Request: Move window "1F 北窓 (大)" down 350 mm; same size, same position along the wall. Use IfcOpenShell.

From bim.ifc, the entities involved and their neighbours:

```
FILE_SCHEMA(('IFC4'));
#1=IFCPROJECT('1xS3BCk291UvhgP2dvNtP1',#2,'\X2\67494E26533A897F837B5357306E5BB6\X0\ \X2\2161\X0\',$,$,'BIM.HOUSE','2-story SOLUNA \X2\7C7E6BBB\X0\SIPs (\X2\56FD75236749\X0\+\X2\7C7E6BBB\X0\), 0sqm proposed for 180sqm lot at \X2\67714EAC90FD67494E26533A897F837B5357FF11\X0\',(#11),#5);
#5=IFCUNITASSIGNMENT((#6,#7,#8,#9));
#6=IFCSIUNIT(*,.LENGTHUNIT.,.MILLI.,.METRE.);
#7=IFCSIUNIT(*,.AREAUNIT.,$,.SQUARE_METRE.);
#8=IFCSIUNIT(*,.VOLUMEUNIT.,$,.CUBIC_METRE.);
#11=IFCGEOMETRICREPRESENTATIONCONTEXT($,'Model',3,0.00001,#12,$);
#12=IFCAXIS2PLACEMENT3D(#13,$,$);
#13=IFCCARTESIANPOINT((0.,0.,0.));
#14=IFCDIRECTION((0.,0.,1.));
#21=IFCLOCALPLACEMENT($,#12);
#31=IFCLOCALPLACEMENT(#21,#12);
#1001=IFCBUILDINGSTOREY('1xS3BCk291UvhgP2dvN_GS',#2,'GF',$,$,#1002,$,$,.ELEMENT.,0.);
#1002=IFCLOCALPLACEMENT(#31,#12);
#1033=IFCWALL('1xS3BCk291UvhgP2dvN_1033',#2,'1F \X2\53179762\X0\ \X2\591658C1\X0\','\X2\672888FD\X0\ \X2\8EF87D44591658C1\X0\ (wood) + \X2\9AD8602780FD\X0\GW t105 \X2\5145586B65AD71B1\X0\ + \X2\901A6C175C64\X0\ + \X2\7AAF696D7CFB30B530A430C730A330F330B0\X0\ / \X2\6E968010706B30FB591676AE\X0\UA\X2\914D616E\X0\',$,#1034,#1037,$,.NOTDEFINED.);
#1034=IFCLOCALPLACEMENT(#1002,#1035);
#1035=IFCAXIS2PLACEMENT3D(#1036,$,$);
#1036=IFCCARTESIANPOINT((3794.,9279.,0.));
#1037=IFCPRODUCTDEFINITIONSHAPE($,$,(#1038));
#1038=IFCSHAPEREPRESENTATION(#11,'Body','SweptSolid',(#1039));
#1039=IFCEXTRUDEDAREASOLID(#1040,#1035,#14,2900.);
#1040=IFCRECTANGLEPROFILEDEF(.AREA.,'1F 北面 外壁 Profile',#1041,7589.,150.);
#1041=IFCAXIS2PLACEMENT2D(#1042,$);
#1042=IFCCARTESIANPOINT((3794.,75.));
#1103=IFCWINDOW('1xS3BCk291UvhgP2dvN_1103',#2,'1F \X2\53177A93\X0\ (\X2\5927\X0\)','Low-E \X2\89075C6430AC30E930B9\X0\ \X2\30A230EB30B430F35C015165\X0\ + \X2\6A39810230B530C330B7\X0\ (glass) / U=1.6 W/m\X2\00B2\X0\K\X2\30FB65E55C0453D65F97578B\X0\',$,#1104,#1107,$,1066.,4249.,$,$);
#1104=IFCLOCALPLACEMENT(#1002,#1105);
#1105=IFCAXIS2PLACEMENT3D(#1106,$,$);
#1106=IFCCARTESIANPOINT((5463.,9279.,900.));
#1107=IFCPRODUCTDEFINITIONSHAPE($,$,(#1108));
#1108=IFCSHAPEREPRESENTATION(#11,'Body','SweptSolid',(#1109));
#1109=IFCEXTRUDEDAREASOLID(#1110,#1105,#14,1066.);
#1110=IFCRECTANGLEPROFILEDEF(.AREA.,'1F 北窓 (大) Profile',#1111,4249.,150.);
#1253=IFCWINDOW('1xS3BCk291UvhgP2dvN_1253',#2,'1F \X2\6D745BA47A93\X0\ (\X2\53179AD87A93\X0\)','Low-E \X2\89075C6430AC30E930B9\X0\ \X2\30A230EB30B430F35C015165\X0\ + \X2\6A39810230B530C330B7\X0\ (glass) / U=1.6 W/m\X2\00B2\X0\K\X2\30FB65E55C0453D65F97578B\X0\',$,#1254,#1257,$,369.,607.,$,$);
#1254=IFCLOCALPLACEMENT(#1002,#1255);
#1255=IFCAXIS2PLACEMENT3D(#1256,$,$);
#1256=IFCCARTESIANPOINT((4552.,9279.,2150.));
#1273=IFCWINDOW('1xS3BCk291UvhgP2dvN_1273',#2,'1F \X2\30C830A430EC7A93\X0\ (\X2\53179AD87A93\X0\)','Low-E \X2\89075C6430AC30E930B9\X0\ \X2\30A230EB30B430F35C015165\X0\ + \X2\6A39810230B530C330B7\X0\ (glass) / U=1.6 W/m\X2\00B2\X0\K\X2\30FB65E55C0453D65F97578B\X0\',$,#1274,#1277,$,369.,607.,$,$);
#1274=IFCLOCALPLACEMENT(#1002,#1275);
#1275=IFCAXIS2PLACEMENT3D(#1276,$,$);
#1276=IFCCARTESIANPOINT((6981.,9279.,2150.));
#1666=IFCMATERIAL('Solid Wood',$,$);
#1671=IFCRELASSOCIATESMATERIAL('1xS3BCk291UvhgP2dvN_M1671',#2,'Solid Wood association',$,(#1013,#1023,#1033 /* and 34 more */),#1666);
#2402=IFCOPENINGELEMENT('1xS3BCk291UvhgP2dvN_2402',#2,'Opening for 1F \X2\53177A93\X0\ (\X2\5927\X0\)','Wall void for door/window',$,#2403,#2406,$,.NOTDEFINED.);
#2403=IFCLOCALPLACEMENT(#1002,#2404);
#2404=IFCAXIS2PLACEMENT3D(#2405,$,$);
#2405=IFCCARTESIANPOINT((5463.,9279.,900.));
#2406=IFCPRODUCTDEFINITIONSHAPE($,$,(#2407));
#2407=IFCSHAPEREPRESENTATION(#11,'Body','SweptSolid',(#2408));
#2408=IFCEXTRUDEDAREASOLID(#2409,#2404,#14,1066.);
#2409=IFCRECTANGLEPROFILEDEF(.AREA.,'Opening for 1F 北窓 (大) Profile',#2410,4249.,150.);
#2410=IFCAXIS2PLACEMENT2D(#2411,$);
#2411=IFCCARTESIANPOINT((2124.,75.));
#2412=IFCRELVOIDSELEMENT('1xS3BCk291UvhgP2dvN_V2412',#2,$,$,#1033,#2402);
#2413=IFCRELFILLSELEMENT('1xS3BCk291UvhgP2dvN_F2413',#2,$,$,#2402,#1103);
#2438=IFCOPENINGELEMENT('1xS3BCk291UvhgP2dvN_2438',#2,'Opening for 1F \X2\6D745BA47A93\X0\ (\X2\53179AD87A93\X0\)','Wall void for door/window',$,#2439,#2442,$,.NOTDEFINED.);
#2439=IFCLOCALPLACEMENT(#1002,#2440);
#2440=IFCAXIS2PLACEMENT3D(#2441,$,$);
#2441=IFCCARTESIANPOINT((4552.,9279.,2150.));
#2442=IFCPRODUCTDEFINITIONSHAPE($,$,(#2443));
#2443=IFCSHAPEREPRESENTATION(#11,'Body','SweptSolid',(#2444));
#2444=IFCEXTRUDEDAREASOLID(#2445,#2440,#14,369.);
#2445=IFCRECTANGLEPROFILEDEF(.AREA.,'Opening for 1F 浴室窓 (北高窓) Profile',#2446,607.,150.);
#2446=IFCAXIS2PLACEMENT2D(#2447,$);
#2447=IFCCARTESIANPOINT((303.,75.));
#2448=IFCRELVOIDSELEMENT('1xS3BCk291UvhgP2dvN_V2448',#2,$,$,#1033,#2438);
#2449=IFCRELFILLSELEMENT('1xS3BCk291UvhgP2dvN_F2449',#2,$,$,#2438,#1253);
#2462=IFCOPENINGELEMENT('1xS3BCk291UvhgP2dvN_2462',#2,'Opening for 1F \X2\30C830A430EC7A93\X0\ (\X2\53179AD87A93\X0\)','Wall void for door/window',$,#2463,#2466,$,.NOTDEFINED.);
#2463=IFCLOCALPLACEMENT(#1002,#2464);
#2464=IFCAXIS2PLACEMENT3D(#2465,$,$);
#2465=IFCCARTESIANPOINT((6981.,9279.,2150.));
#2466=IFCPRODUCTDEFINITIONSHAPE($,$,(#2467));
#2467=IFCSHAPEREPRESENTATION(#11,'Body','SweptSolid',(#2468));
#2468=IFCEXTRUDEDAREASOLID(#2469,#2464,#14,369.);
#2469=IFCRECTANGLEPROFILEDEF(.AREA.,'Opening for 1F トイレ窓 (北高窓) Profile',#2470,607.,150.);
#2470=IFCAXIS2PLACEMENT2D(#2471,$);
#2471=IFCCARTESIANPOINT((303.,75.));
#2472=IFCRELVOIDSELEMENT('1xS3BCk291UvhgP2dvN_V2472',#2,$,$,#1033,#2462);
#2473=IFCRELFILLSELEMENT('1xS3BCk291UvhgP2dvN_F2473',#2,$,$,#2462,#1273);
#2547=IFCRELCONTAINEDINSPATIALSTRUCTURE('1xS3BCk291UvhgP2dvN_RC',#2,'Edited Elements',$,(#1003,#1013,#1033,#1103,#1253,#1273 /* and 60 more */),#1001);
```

```python
import numpy as np
import ifcopenshell
import ifcopenshell.api.geometry
import ifcopenshell.util.placement
import ifcopenshell.util.unit

model = ifcopenshell.open("bim.ifc")
unit_scale = ifcopenshell.util.unit.calculate_unit_scale(model)

window = model.by_guid("1xS3BCk291UvhgP2dvN_1103")
opening = window.FillsVoids[0].RelatingOpeningElement
dz = -0.35 / unit_scale

shift = np.array([0.0, 0.0, dz])
# The window is not placed relative to its opening, so move both.
for product in (opening, window):
    matrix = ifcopenshell.util.placement.get_local_placement(product.ObjectPlacement)
    matrix[:3, 3] += shift
    ifcopenshell.api.geometry.edit_object_placement(model, product=product, matrix=matrix, is_si=False)

print(f"moved by {dz * unit_scale:+.3f} m")

model.write("bim_v2.ifc")
```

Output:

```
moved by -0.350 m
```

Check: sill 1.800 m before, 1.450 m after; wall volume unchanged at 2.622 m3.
